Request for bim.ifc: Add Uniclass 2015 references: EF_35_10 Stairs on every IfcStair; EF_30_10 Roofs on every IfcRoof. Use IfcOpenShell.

First a look at what the model holds.

```python
import ifcopenshell

model = ifcopenshell.open("bim.ifc")
print(model.schema)
print("classifications:", [c.Name for c in model.by_type("IfcClassification")])
for ifc_class in ("IfcDoor", "IfcRoof", "IfcStair", "IfcWall", "IfcWindow"):
    print(ifc_class, len(model.by_type(ifc_class)))
```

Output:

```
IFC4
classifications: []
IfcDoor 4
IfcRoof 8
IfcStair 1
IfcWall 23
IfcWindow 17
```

```python
import ifcopenshell
import ifcopenshell.api.classification

model = ifcopenshell.open("bim.ifc")

system = ifcopenshell.api.classification.add_classification(model, classification="Uniclass 2015")

codes = {
    "IfcStair": ("EF_35_10", "Stairs"),
    "IfcRoof": ("EF_30_10", "Roofs"),
}
for ifc_class, (code, name) in codes.items():
    products = model.by_type(ifc_class)
    ifcopenshell.api.classification.add_reference(
        model, products=products, classification=system, identification=code, name=name
    )
    print(code, len(products))

model.write("bim_updated.ifc")
```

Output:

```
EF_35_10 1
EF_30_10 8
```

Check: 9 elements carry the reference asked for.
